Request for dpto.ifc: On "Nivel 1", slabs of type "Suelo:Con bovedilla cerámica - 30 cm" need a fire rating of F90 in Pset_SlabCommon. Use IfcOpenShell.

First a look at what the model holds.

```python
import ifcopenshell
import ifcopenshell.util.element

model = ifcopenshell.open("dpto.ifc")
print(model.schema)
storey = next(s for s in model.by_type("IfcBuildingStorey") if s.Name == "Nivel 1")
slabs = [e for e in ifcopenshell.util.element.get_decomposition(storey) if e.is_a("IfcSlab")]
seen = {}
for e in slabs:
    element_type = ifcopenshell.util.element.get_type(e)
    key = (element_type.Name if element_type != e and element_type else None, ifcopenshell.util.element.get_pset(e, "Pset_SlabCommon", "FireRating"))
    seen[key] = seen.get(key, 0) + 1
for (name, value), count in sorted(seen.items(), key=str):
    print(count, "x", name, "|", value)
```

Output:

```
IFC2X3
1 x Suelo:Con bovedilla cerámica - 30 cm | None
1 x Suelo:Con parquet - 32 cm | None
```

```python
import ifcopenshell
import ifcopenshell.api.pset
import ifcopenshell.util.element

model = ifcopenshell.open("dpto.ifc")

storey = next(s for s in model.by_type("IfcBuildingStorey") if s.Name == "Nivel 1")
slabs = [e for e in ifcopenshell.util.element.get_decomposition(storey) if e.is_a("IfcSlab")]

count = 0
for e in slabs:
    element_type = ifcopenshell.util.element.get_type(e)
    if element_type in (None, e) or element_type.Name != "Suelo:Con bovedilla cerámica - 30 cm":
        continue
    # add_pset returns the element's existing set when there is one.
    pset = ifcopenshell.api.pset.add_pset(model, product=e, name="Pset_SlabCommon")
    ifcopenshell.api.pset.edit_pset(model, pset=pset, properties={"FireRating": "F90"})
    count += 1

print(count, "slabs updated")

model.write("dpto_updated.ifc")
```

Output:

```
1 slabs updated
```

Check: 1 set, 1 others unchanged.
